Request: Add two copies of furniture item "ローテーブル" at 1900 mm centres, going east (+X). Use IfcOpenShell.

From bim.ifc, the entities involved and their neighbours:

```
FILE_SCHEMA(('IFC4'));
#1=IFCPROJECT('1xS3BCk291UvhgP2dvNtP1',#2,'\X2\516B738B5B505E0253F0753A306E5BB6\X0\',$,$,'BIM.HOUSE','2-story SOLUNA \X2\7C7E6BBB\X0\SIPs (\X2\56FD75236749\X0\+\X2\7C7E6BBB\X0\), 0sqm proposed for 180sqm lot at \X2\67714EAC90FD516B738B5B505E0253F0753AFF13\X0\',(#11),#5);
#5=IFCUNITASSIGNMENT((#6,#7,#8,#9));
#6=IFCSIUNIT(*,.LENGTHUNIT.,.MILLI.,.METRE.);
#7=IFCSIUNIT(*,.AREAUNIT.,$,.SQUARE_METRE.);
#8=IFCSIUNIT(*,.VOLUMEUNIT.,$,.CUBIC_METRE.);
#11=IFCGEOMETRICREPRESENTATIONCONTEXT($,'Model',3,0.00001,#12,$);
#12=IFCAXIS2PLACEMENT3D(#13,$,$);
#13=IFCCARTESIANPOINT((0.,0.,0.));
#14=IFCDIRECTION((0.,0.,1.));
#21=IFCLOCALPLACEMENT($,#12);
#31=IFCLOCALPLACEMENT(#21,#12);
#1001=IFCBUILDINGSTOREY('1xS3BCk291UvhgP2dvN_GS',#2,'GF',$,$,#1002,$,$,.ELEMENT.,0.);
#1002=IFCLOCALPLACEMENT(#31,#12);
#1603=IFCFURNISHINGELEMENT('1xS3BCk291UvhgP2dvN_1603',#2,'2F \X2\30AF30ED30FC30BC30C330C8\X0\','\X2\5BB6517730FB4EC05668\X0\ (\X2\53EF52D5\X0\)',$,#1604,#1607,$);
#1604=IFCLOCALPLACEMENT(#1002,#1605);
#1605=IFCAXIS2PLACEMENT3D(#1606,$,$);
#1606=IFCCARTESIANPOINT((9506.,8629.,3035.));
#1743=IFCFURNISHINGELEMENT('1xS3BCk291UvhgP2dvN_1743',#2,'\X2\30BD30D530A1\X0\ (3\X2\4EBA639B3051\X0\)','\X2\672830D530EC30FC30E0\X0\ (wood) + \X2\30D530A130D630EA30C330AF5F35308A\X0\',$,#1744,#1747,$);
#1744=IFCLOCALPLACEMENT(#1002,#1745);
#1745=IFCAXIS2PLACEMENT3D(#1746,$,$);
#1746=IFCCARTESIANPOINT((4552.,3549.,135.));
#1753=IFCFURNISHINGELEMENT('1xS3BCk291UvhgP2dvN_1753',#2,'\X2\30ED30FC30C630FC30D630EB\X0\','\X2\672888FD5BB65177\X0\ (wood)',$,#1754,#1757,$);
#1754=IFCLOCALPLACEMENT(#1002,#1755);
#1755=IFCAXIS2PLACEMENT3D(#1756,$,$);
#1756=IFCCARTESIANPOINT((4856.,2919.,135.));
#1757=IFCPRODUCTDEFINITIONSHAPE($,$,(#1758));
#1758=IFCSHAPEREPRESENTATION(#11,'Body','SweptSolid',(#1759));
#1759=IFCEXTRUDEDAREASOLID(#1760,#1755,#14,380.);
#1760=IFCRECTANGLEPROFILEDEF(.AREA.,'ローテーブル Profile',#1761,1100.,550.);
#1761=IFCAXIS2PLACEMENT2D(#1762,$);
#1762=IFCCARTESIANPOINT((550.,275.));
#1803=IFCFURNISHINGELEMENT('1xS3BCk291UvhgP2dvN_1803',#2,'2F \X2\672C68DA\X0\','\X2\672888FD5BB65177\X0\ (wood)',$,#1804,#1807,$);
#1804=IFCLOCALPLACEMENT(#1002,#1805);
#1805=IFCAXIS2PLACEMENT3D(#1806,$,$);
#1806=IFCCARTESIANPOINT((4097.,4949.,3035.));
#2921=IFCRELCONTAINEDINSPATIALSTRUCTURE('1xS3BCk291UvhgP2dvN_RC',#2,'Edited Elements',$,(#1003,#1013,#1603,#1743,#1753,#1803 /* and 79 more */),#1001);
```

```python
import numpy as np
import ifcopenshell
import ifcopenshell.api.geometry
import ifcopenshell.api.root
import ifcopenshell.util.element
import ifcopenshell.util.placement
import ifcopenshell.util.unit

model = ifcopenshell.open("bim.ifc")
unit_scale = ifcopenshell.util.unit.calculate_unit_scale(model)


def reuse_history(source, copy):
    """copy_class also copies each property set's owner history, people and application; keep the originals."""
    for rel in copy.IsDefinedBy:
        if rel.is_a("IfcRelDefinesByProperties") and (history := rel.RelatingPropertyDefinition.OwnerHistory):
            rel.RelatingPropertyDefinition.OwnerHistory = source.OwnerHistory
            ifcopenshell.util.element.remove_deep2(model, history)


source = model.by_guid("1xS3BCk291UvhgP2dvN_1753")
base = ifcopenshell.util.placement.get_local_placement(source.ObjectPlacement)
step = np.array([1.0, 0.0, 0.0]) * 1.9 / unit_scale

for i in range(1, 3):
    copy = ifcopenshell.api.root.copy_class(model, product=source)
    copy.Representation = ifcopenshell.util.element.copy_deep(
        model, source.Representation, exclude=["IfcGeometricRepresentationContext", "IfcRepresentationMap"]
    )
    reuse_history(source, copy)
    matrix = base.copy()
    matrix[:3, 3] += i * step
    print("added at", matrix[:3, 3].round(3) + 0.0)
    ifcopenshell.api.geometry.edit_object_placement(model, product=copy, matrix=matrix, is_si=False)

model.write("bim_v2.ifc")
```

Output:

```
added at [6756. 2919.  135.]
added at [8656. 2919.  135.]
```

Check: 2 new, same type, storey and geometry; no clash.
